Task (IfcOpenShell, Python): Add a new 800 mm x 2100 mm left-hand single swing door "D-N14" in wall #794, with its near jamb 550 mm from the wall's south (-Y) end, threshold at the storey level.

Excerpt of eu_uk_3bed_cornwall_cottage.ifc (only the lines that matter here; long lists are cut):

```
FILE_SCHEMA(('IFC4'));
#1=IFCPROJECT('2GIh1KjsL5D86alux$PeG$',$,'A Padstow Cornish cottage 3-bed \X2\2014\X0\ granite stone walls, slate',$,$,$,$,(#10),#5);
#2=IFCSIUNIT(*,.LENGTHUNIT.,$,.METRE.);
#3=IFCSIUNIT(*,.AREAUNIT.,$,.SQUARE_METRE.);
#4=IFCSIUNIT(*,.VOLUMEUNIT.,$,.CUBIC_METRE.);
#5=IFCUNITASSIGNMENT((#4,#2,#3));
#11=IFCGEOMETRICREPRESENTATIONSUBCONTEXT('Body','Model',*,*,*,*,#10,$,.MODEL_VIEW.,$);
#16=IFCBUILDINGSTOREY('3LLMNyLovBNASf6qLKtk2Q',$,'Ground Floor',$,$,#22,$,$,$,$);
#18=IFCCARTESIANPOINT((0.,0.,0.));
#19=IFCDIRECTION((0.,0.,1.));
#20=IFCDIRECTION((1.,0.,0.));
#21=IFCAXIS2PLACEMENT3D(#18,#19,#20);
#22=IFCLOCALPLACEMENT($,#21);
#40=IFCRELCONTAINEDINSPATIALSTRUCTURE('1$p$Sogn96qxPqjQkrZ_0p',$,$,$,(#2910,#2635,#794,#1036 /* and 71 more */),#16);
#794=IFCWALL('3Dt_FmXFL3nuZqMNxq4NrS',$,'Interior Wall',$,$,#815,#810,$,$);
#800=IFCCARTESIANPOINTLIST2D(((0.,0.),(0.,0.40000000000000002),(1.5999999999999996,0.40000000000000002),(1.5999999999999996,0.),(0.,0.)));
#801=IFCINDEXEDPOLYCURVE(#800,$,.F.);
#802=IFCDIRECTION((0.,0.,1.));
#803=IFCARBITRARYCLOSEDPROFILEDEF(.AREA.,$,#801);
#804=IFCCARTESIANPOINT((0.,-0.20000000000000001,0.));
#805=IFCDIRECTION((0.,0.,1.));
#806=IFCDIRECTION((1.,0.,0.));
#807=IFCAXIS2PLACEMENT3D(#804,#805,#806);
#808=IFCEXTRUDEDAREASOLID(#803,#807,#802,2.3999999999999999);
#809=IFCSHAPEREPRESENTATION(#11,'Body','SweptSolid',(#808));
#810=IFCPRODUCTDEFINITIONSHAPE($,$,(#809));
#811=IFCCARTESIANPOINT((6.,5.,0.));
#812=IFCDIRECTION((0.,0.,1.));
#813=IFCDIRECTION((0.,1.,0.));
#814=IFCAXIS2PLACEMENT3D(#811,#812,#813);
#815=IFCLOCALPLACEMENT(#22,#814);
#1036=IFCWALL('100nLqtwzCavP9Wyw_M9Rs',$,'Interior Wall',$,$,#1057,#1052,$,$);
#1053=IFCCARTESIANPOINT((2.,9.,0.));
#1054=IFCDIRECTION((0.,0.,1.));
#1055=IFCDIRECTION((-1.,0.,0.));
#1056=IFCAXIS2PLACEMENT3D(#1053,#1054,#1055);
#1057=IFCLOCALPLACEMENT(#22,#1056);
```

```python
import numpy as np
import ifcopenshell
import ifcopenshell.api.feature
import ifcopenshell.api.geometry
import ifcopenshell.api.root
import ifcopenshell.api.spatial
import ifcopenshell.geom
import ifcopenshell.util.element
import ifcopenshell.util.placement
import ifcopenshell.util.representation
import ifcopenshell.util.shape
import ifcopenshell.util.unit

model = ifcopenshell.open("eu_uk_3bed_cornwall_cottage.ifc")
unit_scale = ifcopenshell.util.unit.calculate_unit_scale(model)
settings = ifcopenshell.geom.settings()


def volume(element):
    """Net volume in cubic metres, openings subtracted."""
    shape = ifcopenshell.geom.create_shape(settings, element)
    return ifcopenshell.util.shape.get_volume(shape.geometry)


wall = model.by_guid("3Dt_FmXFL3nuZqMNxq4NrS")
storey = ifcopenshell.util.element.get_container(wall, ifc_class="IfcBuildingStorey")
context = ifcopenshell.util.representation.get_context(model, "Model", "Body", "MODEL_VIEW")
before = volume(wall)

width, height, from_end, sill = 0.8, 2.1, 0.55, 0.0  # metres

# The wall runs along its own X axis, and the end named is its -X end.
wall_shape = ifcopenshell.geom.create_shape(settings, wall)
x, y, z = ifcopenshell.util.shape.get_vertices(wall_shape.geometry).T
start = x.min() + from_end
face, thickness = float(y.min()), float(y.max() - y.min())
wall_matrix = ifcopenshell.util.placement.get_local_placement(wall.ObjectPlacement)
level = ifcopenshell.util.placement.get_local_placement(storey.ObjectPlacement)[2, 3]


def in_wall(x, y):
    """Placement at x, y metres in the wall's axes, at sill height."""
    matrix = wall_matrix.copy()
    matrix[:, 3] = wall_matrix @ np.array([x / unit_scale, y / unit_scale, 0.0, 1.0])
    matrix[2, 3] = level + sill / unit_scale
    return matrix


# Opening: a box that overshoots both wall faces by 50 mm.
opening = ifcopenshell.api.root.create_entity(model, ifc_class="IfcOpeningElement", predefined_type="OPENING")
box = ifcopenshell.api.geometry.add_wall_representation(
    model, context=context, length=width, height=height, thickness=thickness + 0.1
)
ifcopenshell.api.geometry.assign_representation(model, product=opening, representation=box)
ifcopenshell.api.geometry.edit_object_placement(model, product=opening, matrix=in_wall(start, face - 0.05), is_si=False)
ifcopenshell.api.feature.add_feature(model, feature=opening, element=wall)

door = ifcopenshell.api.root.create_entity(model, ifc_class="IfcDoor", name="D-N14", predefined_type="DOOR")
door.OverallWidth, door.OverallHeight = width / unit_scale, height / unit_scale
door.OperationType = "SINGLE_SWING_LEFT"
body = ifcopenshell.api.geometry.add_door_representation(
    model,
    context=context,
    overall_width=door.OverallWidth,
    overall_height=door.OverallHeight,
    operation_type="SINGLE_SWING_LEFT",
    lining_properties={"LiningDepth": thickness / unit_scale, "ThresholdDepth": thickness / unit_scale},
)
ifcopenshell.api.geometry.assign_representation(model, product=door, representation=body)
ifcopenshell.api.spatial.assign_container(model, products=[door], relating_structure=storey)
ifcopenshell.api.feature.add_filling(model, opening=opening, element=door)

# The lining spans the wall, so the door starts at the wall face.
ifcopenshell.api.geometry.edit_object_placement(model, product=door, matrix=in_wall(start, face), is_si=False)

after = volume(wall)

print(f"wall volume {before:.3f} -> {after:.3f} m3")

model.write("eu_uk_3bed_cornwall_cottage_rev.ifc")
```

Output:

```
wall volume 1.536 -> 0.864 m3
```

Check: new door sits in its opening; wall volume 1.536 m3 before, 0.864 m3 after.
